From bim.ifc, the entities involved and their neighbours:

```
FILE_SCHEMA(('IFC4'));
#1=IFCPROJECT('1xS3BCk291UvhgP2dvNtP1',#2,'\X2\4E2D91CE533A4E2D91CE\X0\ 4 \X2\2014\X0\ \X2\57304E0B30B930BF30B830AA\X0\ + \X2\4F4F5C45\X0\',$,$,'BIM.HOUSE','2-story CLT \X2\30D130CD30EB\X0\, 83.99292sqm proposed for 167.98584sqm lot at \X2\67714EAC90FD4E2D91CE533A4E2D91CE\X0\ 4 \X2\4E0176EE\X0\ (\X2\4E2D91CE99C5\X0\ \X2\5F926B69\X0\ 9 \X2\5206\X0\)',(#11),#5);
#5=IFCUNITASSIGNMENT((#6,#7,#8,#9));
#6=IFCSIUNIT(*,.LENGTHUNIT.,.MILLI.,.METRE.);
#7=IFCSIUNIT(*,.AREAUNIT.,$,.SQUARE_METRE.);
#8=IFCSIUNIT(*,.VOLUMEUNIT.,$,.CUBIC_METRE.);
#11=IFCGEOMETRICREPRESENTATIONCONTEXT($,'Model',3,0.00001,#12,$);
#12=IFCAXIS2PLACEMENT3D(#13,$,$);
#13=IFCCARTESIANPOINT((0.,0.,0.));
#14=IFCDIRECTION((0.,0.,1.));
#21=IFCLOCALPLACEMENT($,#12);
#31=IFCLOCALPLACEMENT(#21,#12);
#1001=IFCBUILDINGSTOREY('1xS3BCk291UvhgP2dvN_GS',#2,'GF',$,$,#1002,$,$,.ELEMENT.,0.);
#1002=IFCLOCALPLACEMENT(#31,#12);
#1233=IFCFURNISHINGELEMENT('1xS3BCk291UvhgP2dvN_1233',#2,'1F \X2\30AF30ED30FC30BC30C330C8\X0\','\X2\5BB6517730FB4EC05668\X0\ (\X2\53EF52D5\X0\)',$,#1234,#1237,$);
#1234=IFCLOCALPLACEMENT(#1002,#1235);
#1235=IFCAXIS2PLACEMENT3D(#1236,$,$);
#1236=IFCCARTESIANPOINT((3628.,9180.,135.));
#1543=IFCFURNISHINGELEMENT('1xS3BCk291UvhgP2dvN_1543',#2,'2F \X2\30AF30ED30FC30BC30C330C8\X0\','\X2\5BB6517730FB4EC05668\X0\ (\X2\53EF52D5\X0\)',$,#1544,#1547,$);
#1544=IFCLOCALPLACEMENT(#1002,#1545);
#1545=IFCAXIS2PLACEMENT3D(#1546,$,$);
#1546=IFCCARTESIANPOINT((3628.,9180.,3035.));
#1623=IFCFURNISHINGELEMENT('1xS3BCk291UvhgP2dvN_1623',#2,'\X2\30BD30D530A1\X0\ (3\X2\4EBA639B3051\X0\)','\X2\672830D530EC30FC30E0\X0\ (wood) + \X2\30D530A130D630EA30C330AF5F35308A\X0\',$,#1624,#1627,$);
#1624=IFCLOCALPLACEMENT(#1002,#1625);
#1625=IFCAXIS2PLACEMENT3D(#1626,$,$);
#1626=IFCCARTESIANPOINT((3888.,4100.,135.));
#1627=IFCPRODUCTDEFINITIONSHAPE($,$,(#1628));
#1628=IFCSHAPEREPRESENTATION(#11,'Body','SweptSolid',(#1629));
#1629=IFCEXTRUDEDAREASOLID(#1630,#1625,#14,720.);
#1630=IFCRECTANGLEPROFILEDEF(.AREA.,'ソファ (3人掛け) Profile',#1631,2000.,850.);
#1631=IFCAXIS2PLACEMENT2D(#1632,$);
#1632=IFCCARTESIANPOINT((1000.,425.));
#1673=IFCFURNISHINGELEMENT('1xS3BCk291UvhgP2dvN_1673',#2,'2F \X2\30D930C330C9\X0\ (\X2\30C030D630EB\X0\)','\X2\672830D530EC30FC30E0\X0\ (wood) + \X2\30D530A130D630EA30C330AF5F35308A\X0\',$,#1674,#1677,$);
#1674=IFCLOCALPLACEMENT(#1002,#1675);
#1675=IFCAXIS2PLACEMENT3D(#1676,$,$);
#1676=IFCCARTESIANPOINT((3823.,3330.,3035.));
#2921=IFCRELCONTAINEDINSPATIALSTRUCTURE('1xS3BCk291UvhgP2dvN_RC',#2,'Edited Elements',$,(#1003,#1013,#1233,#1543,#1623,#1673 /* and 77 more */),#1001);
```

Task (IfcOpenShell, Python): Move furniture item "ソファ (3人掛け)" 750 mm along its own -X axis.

```python
import ifcopenshell
import ifcopenshell.api.geometry
import ifcopenshell.util.placement

model = ifcopenshell.open("bim.ifc")

item = model.by_guid("1xS3BCk291UvhgP2dvN_1623")
matrix = ifcopenshell.util.placement.get_local_placement(item.ObjectPlacement)
matrix[:3, 3] -= matrix[:3, 0] * 750.0
ifcopenshell.api.geometry.edit_object_placement(model, product=item, matrix=matrix, is_si=False)

print(ifcopenshell.util.placement.get_local_placement(item.ObjectPlacement).round(3) + 0.0)

model.write("bim_edited.ifc")
```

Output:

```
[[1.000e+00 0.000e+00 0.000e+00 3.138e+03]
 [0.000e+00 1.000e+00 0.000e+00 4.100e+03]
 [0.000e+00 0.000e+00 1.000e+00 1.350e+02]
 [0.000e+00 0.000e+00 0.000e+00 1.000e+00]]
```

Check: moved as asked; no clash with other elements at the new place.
